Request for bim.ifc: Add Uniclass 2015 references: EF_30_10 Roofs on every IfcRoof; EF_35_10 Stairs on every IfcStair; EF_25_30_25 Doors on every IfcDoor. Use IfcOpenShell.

First a look at what the model holds.

```python
import ifcopenshell

model = ifcopenshell.open("bim.ifc")
print(model.schema)
print("classifications:", [c.Name for c in model.by_type("IfcClassification")])
for ifc_class in ("IfcDoor", "IfcRoof", "IfcStair", "IfcWall", "IfcWindow"):
    print(ifc_class, len(model.by_type(ifc_class)))
```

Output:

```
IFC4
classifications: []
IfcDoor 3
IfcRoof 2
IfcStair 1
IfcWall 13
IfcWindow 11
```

```python
import ifcopenshell
import ifcopenshell.api.classification

model = ifcopenshell.open("bim.ifc")

system = ifcopenshell.api.classification.add_classification(model, classification="Uniclass 2015")

codes = {
    "IfcRoof": ("EF_30_10", "Roofs"),
    "IfcStair": ("EF_35_10", "Stairs"),
    "IfcDoor": ("EF_25_30_25", "Doors"),
}
for ifc_class, (code, name) in codes.items():
    products = model.by_type(ifc_class)
    ifcopenshell.api.classification.add_reference(
        model, products=products, classification=system, identification=code, name=name
    )
    print(code, len(products))

model.write("bim_edited.ifc")
```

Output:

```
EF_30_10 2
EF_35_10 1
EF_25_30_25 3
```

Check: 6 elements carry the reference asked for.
